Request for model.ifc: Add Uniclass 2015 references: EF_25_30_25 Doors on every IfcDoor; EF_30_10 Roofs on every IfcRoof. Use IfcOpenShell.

First a look at what the model holds.

```python
import ifcopenshell

model = ifcopenshell.open("model.ifc")
print(model.schema)
print("classifications:", [c.Name for c in model.by_type("IfcClassification")])
for ifc_class in ("IfcDoor", "IfcRoof", "IfcStair", "IfcWall", "IfcWindow"):
    print(ifc_class, len(model.by_type(ifc_class)))
```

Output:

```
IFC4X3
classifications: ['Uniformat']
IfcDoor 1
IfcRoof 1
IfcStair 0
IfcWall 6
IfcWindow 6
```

```python
import ifcopenshell
import ifcopenshell.api.classification

model = ifcopenshell.open("model.ifc")

system = ifcopenshell.api.classification.add_classification(model, classification="Uniclass 2015")

codes = {
    "IfcDoor": ("EF_25_30_25", "Doors"),
    "IfcRoof": ("EF_30_10", "Roofs"),
}
for ifc_class, (code, name) in codes.items():
    products = model.by_type(ifc_class)
    ifcopenshell.api.classification.add_reference(
        model, products=products, classification=system, identification=code, name=name
    )
    print(code, len(products))

model.write("model_rev.ifc")
```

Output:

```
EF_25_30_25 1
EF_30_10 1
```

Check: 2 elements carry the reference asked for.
